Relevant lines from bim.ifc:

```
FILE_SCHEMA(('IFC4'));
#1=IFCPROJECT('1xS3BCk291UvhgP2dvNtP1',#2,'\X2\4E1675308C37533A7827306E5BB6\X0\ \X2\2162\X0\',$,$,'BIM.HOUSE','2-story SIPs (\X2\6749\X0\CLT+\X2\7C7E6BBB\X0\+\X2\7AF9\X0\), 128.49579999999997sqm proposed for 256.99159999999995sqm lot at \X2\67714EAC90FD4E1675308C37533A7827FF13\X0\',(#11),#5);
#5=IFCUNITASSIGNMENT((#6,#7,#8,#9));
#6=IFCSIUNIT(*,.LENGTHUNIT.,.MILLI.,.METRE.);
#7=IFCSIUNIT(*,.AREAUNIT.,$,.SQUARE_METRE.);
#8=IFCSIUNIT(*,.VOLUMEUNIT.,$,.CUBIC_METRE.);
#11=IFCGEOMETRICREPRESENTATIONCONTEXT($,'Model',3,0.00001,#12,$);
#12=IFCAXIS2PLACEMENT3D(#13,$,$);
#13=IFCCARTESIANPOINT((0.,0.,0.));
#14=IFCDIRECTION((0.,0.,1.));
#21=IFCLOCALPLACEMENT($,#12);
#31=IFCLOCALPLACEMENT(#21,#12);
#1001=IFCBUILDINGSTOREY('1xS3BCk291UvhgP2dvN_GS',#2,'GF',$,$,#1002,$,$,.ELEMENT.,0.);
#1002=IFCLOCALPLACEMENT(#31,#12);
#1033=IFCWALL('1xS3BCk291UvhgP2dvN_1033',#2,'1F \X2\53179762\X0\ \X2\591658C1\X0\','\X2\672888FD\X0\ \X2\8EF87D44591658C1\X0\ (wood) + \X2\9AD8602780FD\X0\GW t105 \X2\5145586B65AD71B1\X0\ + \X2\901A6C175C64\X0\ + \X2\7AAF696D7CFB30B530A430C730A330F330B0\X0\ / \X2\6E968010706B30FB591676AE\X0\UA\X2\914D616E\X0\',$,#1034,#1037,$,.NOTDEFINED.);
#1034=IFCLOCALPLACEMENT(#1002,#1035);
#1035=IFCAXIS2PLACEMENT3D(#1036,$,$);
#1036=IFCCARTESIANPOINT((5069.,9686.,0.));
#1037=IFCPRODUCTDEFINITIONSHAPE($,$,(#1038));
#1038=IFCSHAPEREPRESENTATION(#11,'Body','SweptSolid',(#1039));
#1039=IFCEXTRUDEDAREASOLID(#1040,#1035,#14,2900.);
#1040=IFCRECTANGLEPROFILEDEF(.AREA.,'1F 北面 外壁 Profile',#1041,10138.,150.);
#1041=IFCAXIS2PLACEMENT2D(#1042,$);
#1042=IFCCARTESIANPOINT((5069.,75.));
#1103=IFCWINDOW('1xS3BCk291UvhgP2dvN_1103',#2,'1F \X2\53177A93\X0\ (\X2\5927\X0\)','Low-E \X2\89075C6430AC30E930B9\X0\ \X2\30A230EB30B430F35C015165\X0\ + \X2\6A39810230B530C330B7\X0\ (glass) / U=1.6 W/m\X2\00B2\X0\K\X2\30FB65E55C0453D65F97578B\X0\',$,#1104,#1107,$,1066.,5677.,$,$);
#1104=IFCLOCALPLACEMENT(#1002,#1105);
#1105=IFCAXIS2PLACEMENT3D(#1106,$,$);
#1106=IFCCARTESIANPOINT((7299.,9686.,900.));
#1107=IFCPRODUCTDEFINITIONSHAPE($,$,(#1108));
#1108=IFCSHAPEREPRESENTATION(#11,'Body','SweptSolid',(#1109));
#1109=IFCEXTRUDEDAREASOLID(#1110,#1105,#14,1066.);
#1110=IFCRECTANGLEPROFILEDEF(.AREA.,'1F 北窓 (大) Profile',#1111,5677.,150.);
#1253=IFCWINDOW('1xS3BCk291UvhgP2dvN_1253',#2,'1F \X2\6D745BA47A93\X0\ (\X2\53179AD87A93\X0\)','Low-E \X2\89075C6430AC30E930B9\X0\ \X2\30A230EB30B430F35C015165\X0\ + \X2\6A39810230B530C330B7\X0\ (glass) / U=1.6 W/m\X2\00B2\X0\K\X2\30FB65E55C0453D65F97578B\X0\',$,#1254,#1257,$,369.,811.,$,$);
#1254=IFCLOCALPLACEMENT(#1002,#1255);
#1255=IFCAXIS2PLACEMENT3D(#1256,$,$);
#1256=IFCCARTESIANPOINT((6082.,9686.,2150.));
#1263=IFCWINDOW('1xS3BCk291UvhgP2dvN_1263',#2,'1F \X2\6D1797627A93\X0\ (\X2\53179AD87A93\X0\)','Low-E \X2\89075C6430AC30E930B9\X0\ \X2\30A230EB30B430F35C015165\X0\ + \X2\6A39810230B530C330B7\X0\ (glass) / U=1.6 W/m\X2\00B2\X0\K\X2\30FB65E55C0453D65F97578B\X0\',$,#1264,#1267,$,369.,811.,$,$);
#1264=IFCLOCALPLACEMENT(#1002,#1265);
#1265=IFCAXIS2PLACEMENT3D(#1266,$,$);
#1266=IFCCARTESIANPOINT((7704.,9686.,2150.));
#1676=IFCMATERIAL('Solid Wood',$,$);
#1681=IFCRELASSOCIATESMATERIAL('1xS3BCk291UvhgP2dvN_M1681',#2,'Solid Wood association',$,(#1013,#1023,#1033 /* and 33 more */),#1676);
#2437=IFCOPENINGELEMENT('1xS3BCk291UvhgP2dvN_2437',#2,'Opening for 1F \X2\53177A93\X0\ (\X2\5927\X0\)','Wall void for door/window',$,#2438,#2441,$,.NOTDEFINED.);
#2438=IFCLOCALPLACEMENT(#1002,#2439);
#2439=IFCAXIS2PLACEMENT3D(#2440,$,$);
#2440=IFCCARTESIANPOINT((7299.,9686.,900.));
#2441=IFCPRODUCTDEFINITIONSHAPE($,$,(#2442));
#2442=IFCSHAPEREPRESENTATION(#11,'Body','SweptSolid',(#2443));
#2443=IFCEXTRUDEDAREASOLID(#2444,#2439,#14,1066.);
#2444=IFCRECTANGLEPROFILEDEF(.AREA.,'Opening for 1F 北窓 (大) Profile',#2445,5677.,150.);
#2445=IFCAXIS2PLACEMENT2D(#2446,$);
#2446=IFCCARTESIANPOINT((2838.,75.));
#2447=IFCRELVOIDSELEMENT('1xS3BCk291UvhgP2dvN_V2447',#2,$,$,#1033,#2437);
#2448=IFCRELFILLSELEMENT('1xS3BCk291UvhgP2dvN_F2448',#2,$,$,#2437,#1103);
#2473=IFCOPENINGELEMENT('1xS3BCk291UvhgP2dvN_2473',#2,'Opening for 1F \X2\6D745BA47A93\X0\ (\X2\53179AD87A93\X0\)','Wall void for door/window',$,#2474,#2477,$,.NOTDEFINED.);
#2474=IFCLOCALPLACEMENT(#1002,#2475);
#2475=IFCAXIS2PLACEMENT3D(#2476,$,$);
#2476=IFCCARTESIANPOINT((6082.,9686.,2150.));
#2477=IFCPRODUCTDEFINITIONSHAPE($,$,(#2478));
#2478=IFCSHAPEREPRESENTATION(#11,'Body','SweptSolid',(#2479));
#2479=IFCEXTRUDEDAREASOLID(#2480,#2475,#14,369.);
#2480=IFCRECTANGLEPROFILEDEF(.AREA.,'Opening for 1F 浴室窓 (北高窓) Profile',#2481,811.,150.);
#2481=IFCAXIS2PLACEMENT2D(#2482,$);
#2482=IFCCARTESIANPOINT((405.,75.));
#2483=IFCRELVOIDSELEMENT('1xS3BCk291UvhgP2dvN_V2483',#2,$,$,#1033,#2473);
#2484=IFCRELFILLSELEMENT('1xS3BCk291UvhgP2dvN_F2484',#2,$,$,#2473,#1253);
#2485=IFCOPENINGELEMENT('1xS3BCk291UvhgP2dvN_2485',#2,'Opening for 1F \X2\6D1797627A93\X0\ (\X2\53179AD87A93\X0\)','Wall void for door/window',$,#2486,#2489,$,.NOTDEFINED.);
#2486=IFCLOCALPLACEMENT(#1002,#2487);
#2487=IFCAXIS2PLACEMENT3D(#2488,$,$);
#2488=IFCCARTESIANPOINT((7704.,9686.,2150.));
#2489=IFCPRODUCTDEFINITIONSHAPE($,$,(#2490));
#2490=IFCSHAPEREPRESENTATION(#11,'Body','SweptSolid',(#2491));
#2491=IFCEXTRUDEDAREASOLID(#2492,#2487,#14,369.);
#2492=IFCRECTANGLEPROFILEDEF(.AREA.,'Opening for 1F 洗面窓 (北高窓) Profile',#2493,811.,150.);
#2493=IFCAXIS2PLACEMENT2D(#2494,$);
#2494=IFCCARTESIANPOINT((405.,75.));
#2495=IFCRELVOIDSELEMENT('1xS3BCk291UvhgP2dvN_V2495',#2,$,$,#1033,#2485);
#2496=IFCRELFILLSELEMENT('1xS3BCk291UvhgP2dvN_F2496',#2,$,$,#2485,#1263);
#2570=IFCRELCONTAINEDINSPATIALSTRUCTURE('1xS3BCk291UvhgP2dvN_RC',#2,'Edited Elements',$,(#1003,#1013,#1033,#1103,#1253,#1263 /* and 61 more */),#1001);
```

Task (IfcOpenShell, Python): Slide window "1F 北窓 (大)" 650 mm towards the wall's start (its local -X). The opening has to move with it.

```python
import ifcopenshell
import ifcopenshell.api.geometry
import ifcopenshell.util.placement
import ifcopenshell.util.unit

model = ifcopenshell.open("bim.ifc")
unit_scale = ifcopenshell.util.unit.calculate_unit_scale(model)

window = model.by_guid("1xS3BCk291UvhgP2dvN_1103")
opening = window.FillsVoids[0].RelatingOpeningElement
wall = opening.VoidsElements[0].RelatingBuildingElement

wall_matrix = ifcopenshell.util.placement.get_local_placement(wall.ObjectPlacement)
shift = wall_matrix[:3, 0] * -0.65 / unit_scale
before = ifcopenshell.util.placement.get_local_placement(window.ObjectPlacement)[:3, 3].copy()

# The window is not placed relative to its opening, so move both.
for product in (opening, window):
    matrix = ifcopenshell.util.placement.get_local_placement(product.ObjectPlacement)
    matrix[:3, 3] += shift
    ifcopenshell.api.geometry.edit_object_placement(model, product=product, matrix=matrix, is_si=False)

after = ifcopenshell.util.placement.get_local_placement(window.ObjectPlacement)[:3, 3]
print("window moved by", (after - before).round(3) + 0.0)

model.write("bim_v2.ifc")
```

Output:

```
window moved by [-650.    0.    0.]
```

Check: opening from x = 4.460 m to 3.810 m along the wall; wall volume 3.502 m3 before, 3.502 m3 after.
